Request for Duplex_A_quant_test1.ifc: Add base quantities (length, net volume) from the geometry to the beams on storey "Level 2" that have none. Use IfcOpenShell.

First a look at what the model holds.

```python
import ifcopenshell
import ifcopenshell.util.element
import ifcopenshell.util.unit

model = ifcopenshell.open("Duplex_A_quant_test1.ifc")
print(model.schema)
for unit_type in ("LENGTHUNIT", "AREAUNIT", "VOLUMEUNIT"):
    print(unit_type, ifcopenshell.util.unit.calculate_unit_scale(model, unit_type))
storey = next(s for s in model.by_type("IfcBuildingStorey") if s.Name == "Level 2")
beams = [e for e in ifcopenshell.util.element.get_decomposition(storey) if e.is_a("IfcBeam")]
for e in sorted(beams, key=lambda e: e.id()):
    print(e.id(), e.is_a(), e.Name, list(ifcopenshell.util.element.get_psets(e, qtos_only=True)), sep=" | ")
```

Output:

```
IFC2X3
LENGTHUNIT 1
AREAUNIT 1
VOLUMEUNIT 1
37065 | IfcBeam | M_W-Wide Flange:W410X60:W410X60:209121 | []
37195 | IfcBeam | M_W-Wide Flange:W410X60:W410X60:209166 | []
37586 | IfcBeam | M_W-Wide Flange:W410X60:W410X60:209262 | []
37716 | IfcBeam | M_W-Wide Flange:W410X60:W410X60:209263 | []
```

```python
import ifcopenshell
import ifcopenshell.api.pset
import ifcopenshell.geom
import ifcopenshell.util.element
import ifcopenshell.util.shape
import ifcopenshell.util.unit

model = ifcopenshell.open("Duplex_A_quant_test1.ifc")
unit_scale = ifcopenshell.util.unit.calculate_unit_scale(model)
volume_scale = ifcopenshell.util.unit.calculate_unit_scale(model, "VOLUMEUNIT")
settings = ifcopenshell.geom.settings()

storey = next(s for s in model.by_type("IfcBuildingStorey") if s.Name == "Level 2")
beams = [e for e in ifcopenshell.util.element.get_decomposition(storey) if e.is_a("IfcBeam")]

for e in sorted(beams, key=lambda e: e.id()):
    if ifcopenshell.util.element.get_psets(e, qtos_only=True, should_inherit=False):
        continue
    # Geometry comes back in metres, in the element's own axes.
    shape = ifcopenshell.geom.create_shape(settings, e)
    values = {
        "Length": ifcopenshell.util.shape.get_max_xyz(shape.geometry) / unit_scale,
        "NetVolume": ifcopenshell.util.shape.get_volume(shape.geometry) / volume_scale,
    }
    qto = ifcopenshell.api.pset.add_qto(model, product=e, name="BaseQuantities")
    ifcopenshell.api.pset.edit_qto(model, qto=qto, properties=values)
    print(e.id(), {k: round(v, 3) for k, v in values.items()})

model.write("Duplex_A_quant_test1-out.ifc")
```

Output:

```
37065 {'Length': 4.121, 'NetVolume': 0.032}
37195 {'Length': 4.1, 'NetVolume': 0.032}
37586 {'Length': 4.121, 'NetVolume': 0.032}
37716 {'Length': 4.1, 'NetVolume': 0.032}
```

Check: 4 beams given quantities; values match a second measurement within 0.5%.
